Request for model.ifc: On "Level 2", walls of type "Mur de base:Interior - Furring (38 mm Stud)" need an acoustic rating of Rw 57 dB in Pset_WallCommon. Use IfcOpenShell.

First a look at what the model holds.

```python
import ifcopenshell
import ifcopenshell.util.element

model = ifcopenshell.open("model.ifc")
print(model.schema)
storey = next(s for s in model.by_type("IfcBuildingStorey") if s.Name == "Level 2")
walls = [e for e in ifcopenshell.util.element.get_decomposition(storey) if e.is_a("IfcWall")]
seen = {}
for e in walls:
    element_type = ifcopenshell.util.element.get_type(e)
    key = (element_type.Name if element_type != e and element_type else None, ifcopenshell.util.element.get_pset(e, "Pset_WallCommon", "AcousticRating"))
    seen[key] = seen.get(key, 0) + 1
for (name, value), count in sorted(seen.items(), key=str):
    print(count, "x", name, "|", value)
```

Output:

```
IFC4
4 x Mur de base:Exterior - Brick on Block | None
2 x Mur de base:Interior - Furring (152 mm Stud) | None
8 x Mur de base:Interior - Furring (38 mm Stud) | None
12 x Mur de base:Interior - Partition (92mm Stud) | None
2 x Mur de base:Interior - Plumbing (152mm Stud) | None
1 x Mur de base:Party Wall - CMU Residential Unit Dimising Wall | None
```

```python
import ifcopenshell
import ifcopenshell.api.pset
import ifcopenshell.util.element

model = ifcopenshell.open("model.ifc")

storey = next(s for s in model.by_type("IfcBuildingStorey") if s.Name == "Level 2")
walls = [e for e in ifcopenshell.util.element.get_decomposition(storey) if e.is_a("IfcWall")]

count = 0
for e in walls:
    element_type = ifcopenshell.util.element.get_type(e)
    if element_type in (None, e) or element_type.Name != "Mur de base:Interior - Furring (38 mm Stud)":
        continue
    # add_pset returns the element's existing set when there is one.
    pset = ifcopenshell.api.pset.add_pset(model, product=e, name="Pset_WallCommon")
    ifcopenshell.api.pset.edit_pset(model, pset=pset, properties={"AcousticRating": "Rw 57 dB"})
    count += 1

print(count, "walls updated")

model.write("model-out.ifc")
```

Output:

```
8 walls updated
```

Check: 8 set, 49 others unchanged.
